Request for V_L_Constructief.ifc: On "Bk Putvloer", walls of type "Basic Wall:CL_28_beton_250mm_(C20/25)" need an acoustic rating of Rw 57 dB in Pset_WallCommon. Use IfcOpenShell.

First a look at what the model holds.

```python
import ifcopenshell
import ifcopenshell.util.element

model = ifcopenshell.open("V_L_Constructief.ifc")
print(model.schema)
storey = next(s for s in model.by_type("IfcBuildingStorey") if s.Name == "Bk Putvloer")
walls = [e for e in ifcopenshell.util.element.get_decomposition(storey) if e.is_a("IfcWall")]
seen = {}
for e in walls:
    element_type = ifcopenshell.util.element.get_type(e)
    key = (element_type.Name if element_type != e and element_type else None, ifcopenshell.util.element.get_pset(e, "Pset_WallCommon", "AcousticRating"))
    seen[key] = seen.get(key, 0) + 1
for (name, value), count in sorted(seen.items(), key=str):
    print(count, "x", name, "|", value)
```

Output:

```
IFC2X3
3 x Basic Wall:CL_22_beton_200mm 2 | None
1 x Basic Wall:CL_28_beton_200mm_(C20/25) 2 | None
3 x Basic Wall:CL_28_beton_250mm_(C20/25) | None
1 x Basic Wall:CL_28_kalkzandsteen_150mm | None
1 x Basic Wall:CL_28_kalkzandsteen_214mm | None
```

```python
import ifcopenshell
import ifcopenshell.api.pset
import ifcopenshell.util.element

model = ifcopenshell.open("V_L_Constructief.ifc")

storey = next(s for s in model.by_type("IfcBuildingStorey") if s.Name == "Bk Putvloer")
walls = [e for e in ifcopenshell.util.element.get_decomposition(storey) if e.is_a("IfcWall")]

count = 0
for e in walls:
    element_type = ifcopenshell.util.element.get_type(e)
    if element_type in (None, e) or element_type.Name != "Basic Wall:CL_28_beton_250mm_(C20/25)":
        continue
    found = ifcopenshell.util.element.get_pset(e, "Pset_WallCommon", should_inherit=False)
    if found:
        pset = model.by_id(found["id"])
        if len(ifcopenshell.util.element.get_elements_by_pset(pset)) > 1:
            pset = ifcopenshell.api.pset.unshare_pset(model, products=[e], pset=pset)[0]
    else:
        pset = ifcopenshell.api.pset.add_pset(model, product=e, name="Pset_WallCommon")
    ifcopenshell.api.pset.edit_pset(model, pset=pset, properties={"AcousticRating": "Rw 57 dB"})
    count += 1

print(count, "walls updated")

model.write("V_L_Constructief_edited.ifc")
```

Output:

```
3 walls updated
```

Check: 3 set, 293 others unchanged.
